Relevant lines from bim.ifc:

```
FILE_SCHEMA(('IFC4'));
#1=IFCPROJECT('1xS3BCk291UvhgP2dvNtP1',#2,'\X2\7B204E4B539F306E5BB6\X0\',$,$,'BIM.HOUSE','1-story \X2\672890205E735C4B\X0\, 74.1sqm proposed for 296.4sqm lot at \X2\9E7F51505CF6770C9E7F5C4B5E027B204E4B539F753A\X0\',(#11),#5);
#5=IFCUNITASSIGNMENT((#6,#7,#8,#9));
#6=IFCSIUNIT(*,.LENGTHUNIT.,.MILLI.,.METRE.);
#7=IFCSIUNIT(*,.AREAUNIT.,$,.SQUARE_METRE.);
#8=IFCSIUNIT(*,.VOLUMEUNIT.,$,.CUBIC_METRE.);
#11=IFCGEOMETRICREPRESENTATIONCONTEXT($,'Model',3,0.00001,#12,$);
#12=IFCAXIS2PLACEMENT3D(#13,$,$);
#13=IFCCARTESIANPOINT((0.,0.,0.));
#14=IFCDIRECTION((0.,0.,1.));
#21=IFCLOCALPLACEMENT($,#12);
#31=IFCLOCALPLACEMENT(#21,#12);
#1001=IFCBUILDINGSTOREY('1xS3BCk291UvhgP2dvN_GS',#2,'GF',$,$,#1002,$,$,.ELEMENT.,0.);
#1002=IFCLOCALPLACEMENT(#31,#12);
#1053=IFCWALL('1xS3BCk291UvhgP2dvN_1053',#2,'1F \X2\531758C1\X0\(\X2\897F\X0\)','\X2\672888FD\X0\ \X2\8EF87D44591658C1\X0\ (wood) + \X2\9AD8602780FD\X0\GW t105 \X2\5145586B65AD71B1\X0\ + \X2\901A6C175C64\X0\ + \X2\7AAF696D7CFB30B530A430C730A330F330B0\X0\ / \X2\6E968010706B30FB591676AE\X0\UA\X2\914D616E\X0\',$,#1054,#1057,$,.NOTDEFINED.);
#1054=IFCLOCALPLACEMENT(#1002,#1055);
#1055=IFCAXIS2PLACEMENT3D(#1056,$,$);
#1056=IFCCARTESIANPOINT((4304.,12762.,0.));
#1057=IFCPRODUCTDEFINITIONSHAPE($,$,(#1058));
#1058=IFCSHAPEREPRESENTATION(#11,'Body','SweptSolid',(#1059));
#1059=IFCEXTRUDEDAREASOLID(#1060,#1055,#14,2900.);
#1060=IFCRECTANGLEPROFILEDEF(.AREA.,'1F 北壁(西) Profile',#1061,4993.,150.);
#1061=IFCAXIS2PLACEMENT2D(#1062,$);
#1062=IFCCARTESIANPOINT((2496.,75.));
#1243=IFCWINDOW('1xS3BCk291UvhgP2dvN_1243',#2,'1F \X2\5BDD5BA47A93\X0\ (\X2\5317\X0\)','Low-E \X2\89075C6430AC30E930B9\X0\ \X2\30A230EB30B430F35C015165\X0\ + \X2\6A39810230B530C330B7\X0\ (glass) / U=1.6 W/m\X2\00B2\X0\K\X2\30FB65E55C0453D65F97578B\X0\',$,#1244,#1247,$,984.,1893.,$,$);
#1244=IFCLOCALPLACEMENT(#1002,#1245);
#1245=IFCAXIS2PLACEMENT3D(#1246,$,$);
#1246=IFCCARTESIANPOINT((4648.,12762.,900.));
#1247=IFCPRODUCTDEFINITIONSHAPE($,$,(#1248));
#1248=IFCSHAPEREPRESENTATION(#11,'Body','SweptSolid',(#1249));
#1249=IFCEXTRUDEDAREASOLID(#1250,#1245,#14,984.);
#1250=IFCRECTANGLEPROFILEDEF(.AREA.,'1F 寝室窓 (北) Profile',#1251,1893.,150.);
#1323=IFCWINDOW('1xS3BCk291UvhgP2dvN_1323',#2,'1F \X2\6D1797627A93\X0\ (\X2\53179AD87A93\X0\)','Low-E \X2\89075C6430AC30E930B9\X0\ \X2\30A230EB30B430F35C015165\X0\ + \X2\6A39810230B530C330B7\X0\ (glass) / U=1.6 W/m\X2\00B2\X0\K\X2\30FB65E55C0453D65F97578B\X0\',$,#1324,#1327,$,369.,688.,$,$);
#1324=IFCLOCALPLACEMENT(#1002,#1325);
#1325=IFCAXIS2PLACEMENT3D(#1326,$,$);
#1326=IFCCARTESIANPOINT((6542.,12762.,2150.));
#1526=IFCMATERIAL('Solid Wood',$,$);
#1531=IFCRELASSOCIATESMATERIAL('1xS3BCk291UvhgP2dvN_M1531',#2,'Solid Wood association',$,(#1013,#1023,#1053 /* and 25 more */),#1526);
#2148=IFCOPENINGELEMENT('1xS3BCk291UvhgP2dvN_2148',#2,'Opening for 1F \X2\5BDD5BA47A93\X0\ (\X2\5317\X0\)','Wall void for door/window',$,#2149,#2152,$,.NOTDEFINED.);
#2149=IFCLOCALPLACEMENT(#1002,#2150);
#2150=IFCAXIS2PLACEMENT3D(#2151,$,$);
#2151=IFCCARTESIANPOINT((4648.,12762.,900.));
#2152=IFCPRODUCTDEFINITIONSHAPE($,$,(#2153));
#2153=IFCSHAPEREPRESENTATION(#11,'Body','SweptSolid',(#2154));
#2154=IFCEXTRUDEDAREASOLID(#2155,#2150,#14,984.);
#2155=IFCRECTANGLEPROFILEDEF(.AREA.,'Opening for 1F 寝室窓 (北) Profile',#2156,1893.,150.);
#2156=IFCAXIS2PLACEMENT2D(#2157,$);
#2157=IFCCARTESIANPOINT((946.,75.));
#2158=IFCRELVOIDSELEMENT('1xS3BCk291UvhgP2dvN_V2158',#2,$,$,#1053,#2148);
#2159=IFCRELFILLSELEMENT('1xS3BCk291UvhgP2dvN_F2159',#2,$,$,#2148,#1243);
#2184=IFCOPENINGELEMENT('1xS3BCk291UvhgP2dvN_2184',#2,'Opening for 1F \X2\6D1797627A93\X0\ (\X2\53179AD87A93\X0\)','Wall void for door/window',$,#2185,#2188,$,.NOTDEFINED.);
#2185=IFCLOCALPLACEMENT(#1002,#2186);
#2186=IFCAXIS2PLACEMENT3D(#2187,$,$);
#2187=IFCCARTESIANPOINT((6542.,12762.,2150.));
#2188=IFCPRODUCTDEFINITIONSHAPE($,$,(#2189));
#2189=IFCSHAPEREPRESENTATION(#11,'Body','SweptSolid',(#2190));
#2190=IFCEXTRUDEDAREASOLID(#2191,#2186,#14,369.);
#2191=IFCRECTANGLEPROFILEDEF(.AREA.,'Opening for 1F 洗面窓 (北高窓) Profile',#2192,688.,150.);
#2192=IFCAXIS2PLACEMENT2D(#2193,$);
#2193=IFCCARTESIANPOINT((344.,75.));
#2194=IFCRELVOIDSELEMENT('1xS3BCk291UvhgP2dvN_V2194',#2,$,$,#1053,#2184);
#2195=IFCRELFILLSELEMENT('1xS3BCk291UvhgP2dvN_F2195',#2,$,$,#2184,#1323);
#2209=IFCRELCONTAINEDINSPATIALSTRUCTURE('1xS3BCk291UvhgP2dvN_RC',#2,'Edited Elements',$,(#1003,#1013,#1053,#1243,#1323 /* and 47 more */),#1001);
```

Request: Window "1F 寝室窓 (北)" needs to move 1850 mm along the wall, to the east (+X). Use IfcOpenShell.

```python
import ifcopenshell
import ifcopenshell.api.geometry
import ifcopenshell.util.placement
import ifcopenshell.util.unit

model = ifcopenshell.open("bim.ifc")
unit_scale = ifcopenshell.util.unit.calculate_unit_scale(model)

window = model.by_guid("1xS3BCk291UvhgP2dvN_1243")
opening = window.FillsVoids[0].RelatingOpeningElement
wall = opening.VoidsElements[0].RelatingBuildingElement

wall_matrix = ifcopenshell.util.placement.get_local_placement(wall.ObjectPlacement)
shift = wall_matrix[:3, 0] * 1.85 / unit_scale
before = ifcopenshell.util.placement.get_local_placement(window.ObjectPlacement)[:3, 3].copy()

# The window is not placed relative to its opening, so move both.
for product in (opening, window):
    matrix = ifcopenshell.util.placement.get_local_placement(product.ObjectPlacement)
    matrix[:3, 3] += shift
    ifcopenshell.api.geometry.edit_object_placement(model, product=product, matrix=matrix, is_si=False)

after = ifcopenshell.util.placement.get_local_placement(window.ObjectPlacement)[:3, 3]
print("window moved by", (after - before).round(3) + 0.0)

model.write("bim_edited.ifc")
```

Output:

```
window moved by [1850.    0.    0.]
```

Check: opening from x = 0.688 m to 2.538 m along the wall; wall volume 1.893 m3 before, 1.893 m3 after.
